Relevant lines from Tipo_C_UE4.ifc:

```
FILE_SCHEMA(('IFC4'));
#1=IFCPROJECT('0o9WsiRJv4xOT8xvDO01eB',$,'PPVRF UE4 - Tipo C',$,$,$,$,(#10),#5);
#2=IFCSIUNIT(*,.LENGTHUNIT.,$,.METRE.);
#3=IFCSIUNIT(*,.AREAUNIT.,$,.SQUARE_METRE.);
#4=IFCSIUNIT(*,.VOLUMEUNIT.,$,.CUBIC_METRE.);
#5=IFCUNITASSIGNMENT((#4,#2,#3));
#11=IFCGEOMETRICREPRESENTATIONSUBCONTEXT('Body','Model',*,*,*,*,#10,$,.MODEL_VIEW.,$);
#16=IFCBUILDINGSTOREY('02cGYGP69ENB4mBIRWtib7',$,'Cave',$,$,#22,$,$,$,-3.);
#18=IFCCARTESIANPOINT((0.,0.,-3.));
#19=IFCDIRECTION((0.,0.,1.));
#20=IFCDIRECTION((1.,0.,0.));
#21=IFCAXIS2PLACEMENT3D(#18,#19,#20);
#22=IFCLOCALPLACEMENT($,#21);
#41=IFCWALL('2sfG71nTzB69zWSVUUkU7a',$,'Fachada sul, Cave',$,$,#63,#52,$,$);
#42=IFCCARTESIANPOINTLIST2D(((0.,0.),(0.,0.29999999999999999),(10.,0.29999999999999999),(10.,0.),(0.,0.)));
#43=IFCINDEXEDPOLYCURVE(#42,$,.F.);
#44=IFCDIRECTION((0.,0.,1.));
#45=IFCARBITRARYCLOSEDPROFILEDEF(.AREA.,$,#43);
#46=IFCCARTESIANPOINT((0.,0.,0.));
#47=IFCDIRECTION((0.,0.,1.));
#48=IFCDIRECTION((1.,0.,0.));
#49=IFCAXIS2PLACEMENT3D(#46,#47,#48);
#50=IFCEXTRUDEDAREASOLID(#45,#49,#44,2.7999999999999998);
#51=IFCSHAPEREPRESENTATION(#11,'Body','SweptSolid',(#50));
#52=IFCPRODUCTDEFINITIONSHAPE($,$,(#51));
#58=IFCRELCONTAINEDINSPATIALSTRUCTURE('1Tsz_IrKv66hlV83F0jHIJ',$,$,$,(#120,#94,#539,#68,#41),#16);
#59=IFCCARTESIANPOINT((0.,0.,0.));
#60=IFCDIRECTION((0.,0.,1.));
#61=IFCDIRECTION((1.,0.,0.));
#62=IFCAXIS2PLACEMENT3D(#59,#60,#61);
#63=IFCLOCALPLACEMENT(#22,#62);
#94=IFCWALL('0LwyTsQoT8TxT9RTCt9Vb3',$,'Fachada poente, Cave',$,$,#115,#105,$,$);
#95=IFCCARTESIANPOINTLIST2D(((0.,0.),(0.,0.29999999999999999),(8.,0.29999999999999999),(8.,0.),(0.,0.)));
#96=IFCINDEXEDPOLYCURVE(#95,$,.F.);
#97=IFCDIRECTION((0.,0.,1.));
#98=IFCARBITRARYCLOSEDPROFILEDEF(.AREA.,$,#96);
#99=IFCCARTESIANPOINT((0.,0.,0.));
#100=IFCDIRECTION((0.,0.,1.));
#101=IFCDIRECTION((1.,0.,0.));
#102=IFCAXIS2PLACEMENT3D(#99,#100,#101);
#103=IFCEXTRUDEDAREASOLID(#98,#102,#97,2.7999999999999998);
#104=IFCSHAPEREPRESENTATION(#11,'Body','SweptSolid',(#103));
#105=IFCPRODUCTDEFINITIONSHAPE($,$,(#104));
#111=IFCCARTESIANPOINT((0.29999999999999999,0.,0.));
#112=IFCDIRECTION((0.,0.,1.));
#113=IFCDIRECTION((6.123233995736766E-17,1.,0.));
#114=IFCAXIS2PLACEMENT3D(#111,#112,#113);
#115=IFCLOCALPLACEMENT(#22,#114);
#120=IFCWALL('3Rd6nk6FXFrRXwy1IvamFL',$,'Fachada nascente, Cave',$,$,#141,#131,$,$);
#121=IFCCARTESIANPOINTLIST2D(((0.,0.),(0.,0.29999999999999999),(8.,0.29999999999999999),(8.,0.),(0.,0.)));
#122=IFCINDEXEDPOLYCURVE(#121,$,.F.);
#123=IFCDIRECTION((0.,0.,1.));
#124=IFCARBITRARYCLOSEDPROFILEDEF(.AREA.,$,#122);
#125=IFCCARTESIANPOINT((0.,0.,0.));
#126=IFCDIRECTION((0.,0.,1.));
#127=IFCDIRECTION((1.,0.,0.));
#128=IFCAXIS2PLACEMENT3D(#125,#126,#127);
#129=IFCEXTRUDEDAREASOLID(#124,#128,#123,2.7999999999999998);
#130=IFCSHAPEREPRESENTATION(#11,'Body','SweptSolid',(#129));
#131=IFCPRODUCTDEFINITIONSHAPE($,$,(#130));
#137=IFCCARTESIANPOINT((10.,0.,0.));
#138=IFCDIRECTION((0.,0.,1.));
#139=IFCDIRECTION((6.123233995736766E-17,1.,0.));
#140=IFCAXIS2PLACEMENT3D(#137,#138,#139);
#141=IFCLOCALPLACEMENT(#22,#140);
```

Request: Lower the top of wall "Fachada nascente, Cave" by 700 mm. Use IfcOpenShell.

```python
import ifcopenshell
import ifcopenshell.geom
import ifcopenshell.util.representation
import ifcopenshell.util.shape

model = ifcopenshell.open("Tipo_C_UE4.ifc")
settings = ifcopenshell.geom.settings()


def volume(element):
    """Net volume in cubic metres, openings subtracted."""
    shape = ifcopenshell.geom.create_shape(settings, element)
    return ifcopenshell.util.shape.get_volume(shape.geometry)


wall = model.by_guid("3Rd6nk6FXFrRXwy1IvamFL")
before = volume(wall)

body = ifcopenshell.util.representation.get_representation(wall, "Model", "Body")
solid = body.Items[0]
old_height = solid.Depth
solid.Depth -= 0.7
after = volume(wall)

print(f"height {old_height:g} -> {solid.Depth:g}, volume {before:.3f} -> {after:.3f} m3")

model.write("Tipo_C_UE4_updated.ifc")
```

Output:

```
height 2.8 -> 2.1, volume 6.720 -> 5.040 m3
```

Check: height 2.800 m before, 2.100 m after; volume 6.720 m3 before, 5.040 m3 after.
